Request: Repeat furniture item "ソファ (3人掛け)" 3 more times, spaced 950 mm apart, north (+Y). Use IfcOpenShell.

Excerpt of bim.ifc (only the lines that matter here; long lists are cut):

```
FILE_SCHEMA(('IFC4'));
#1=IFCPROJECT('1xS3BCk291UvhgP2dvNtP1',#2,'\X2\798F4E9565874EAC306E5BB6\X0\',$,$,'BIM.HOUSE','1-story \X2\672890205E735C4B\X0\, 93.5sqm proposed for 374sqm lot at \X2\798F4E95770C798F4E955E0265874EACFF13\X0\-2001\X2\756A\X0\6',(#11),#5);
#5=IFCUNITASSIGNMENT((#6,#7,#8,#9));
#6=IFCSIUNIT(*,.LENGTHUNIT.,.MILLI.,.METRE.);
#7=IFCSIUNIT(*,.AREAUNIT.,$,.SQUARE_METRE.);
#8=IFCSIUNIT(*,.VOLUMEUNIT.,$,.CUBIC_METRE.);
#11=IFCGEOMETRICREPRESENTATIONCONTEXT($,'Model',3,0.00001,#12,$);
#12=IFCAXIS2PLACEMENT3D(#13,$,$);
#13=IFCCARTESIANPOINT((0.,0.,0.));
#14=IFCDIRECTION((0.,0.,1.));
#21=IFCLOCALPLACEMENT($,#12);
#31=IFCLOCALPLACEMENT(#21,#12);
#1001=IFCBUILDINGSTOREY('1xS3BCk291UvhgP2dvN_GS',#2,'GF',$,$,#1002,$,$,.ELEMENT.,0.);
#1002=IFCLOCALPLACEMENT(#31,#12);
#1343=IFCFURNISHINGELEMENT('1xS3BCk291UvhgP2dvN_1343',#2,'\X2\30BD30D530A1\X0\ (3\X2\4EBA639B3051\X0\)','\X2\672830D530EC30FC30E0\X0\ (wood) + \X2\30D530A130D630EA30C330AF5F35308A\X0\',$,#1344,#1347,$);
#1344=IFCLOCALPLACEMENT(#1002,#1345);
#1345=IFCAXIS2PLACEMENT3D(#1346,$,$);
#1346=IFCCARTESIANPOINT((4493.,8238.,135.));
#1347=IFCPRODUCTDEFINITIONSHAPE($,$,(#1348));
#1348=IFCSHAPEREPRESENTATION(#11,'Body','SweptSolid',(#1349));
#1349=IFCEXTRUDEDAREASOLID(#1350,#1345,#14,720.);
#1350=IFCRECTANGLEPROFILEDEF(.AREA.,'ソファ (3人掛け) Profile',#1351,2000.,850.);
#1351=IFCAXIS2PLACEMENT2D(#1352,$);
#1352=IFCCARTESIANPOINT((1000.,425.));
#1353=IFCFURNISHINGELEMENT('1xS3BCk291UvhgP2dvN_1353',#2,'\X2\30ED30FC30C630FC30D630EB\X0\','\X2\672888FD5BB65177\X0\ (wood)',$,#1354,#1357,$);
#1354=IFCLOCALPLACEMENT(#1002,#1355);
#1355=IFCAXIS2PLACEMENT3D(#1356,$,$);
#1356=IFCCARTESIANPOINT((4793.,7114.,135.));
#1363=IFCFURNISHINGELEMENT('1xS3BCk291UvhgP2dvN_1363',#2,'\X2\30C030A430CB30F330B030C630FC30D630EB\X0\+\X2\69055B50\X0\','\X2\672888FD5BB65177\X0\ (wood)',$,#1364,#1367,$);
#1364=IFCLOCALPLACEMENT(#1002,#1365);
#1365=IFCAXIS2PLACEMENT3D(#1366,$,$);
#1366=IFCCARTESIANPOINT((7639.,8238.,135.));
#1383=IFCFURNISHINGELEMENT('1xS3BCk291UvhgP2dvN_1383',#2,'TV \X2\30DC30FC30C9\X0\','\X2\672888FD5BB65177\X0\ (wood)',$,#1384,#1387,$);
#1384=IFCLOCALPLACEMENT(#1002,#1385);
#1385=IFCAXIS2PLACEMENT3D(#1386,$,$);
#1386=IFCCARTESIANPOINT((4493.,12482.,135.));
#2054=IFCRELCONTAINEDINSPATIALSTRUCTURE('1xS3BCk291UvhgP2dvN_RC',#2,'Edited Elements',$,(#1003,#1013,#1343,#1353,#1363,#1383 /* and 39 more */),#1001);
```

```python
import numpy as np
import ifcopenshell
import ifcopenshell.api.geometry
import ifcopenshell.api.root
import ifcopenshell.util.element
import ifcopenshell.util.placement

model = ifcopenshell.open("bim.ifc")


def reuse_history(source, copy):
    """copy_class also copies each property set's owner history, people and application; keep the originals."""
    for rel in copy.IsDefinedBy:
        if rel.is_a("IfcRelDefinesByProperties") and (history := rel.RelatingPropertyDefinition.OwnerHistory):
            rel.RelatingPropertyDefinition.OwnerHistory = source.OwnerHistory
            ifcopenshell.util.element.remove_deep2(model, history)


source = model.by_guid("1xS3BCk291UvhgP2dvN_1343")
base = ifcopenshell.util.placement.get_local_placement(source.ObjectPlacement)
step = np.array([0.0, 1.0, 0.0]) * 950.0

for i in range(1, 4):
    copy = ifcopenshell.api.root.copy_class(model, product=source)
    copy.Representation = ifcopenshell.util.element.copy_deep(
        model, source.Representation, exclude=["IfcGeometricRepresentationContext", "IfcRepresentationMap"]
    )
    reuse_history(source, copy)
    matrix = base.copy()
    matrix[:3, 3] += i * step
    print("added at", matrix[:3, 3].round(3) + 0.0)
    ifcopenshell.api.geometry.edit_object_placement(model, product=copy, matrix=matrix, is_si=False)

model.write("bim_rev.ifc")
```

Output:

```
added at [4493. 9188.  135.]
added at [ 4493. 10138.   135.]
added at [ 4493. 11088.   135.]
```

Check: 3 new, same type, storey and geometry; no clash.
